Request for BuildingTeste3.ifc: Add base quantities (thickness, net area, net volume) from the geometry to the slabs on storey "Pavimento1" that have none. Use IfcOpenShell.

First a look at what the model holds.

```python
import ifcopenshell
import ifcopenshell.util.element
import ifcopenshell.util.unit

model = ifcopenshell.open("BuildingTeste3.ifc")
print(model.schema)
for unit_type in ("LENGTHUNIT", "AREAUNIT", "VOLUMEUNIT"):
    print(unit_type, ifcopenshell.util.unit.calculate_unit_scale(model, unit_type))
storey = next(s for s in model.by_type("IfcBuildingStorey") if s.Name == "Pavimento1")
slabs = [e for e in ifcopenshell.util.element.get_decomposition(storey) if e.is_a("IfcSlab")]
for e in sorted(slabs, key=lambda e: e.id()):
    print(e.id(), e.is_a(), e.Name, list(ifcopenshell.util.element.get_psets(e, qtos_only=True)), sep=" | ")
```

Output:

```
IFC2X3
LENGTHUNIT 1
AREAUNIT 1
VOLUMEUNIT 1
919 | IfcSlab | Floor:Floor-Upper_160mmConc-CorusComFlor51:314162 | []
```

```python
import ifcopenshell
import ifcopenshell.api.pset
import ifcopenshell.geom
import ifcopenshell.util.element
import ifcopenshell.util.shape
import ifcopenshell.util.unit

model = ifcopenshell.open("BuildingTeste3.ifc")
unit_scale = ifcopenshell.util.unit.calculate_unit_scale(model)
area_scale = ifcopenshell.util.unit.calculate_unit_scale(model, "AREAUNIT")
volume_scale = ifcopenshell.util.unit.calculate_unit_scale(model, "VOLUMEUNIT")
settings = ifcopenshell.geom.settings()

storey = next(s for s in model.by_type("IfcBuildingStorey") if s.Name == "Pavimento1")
slabs = [e for e in ifcopenshell.util.element.get_decomposition(storey) if e.is_a("IfcSlab")]

for e in sorted(slabs, key=lambda e: e.id()):
    if ifcopenshell.util.element.get_psets(e, qtos_only=True, should_inherit=False):
        continue
    # Geometry comes back in metres, in the element's own axes.
    shape = ifcopenshell.geom.create_shape(settings, e)
    values = {
        "Width": ifcopenshell.util.shape.get_z(shape.geometry) / unit_scale,
        "NetArea": ifcopenshell.util.shape.get_footprint_area(shape.geometry) / area_scale,
        "NetVolume": ifcopenshell.util.shape.get_volume(shape.geometry) / volume_scale,
    }
    qto = ifcopenshell.api.pset.add_qto(model, product=e, name="BaseQuantities")
    ifcopenshell.api.pset.edit_qto(model, qto=qto, properties=values)
    print(e.id(), {k: round(v, 3) for k, v in values.items()})

model.write("BuildingTeste3_rev.ifc")
```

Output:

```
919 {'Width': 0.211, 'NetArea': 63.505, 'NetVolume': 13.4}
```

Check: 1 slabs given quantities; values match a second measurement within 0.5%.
